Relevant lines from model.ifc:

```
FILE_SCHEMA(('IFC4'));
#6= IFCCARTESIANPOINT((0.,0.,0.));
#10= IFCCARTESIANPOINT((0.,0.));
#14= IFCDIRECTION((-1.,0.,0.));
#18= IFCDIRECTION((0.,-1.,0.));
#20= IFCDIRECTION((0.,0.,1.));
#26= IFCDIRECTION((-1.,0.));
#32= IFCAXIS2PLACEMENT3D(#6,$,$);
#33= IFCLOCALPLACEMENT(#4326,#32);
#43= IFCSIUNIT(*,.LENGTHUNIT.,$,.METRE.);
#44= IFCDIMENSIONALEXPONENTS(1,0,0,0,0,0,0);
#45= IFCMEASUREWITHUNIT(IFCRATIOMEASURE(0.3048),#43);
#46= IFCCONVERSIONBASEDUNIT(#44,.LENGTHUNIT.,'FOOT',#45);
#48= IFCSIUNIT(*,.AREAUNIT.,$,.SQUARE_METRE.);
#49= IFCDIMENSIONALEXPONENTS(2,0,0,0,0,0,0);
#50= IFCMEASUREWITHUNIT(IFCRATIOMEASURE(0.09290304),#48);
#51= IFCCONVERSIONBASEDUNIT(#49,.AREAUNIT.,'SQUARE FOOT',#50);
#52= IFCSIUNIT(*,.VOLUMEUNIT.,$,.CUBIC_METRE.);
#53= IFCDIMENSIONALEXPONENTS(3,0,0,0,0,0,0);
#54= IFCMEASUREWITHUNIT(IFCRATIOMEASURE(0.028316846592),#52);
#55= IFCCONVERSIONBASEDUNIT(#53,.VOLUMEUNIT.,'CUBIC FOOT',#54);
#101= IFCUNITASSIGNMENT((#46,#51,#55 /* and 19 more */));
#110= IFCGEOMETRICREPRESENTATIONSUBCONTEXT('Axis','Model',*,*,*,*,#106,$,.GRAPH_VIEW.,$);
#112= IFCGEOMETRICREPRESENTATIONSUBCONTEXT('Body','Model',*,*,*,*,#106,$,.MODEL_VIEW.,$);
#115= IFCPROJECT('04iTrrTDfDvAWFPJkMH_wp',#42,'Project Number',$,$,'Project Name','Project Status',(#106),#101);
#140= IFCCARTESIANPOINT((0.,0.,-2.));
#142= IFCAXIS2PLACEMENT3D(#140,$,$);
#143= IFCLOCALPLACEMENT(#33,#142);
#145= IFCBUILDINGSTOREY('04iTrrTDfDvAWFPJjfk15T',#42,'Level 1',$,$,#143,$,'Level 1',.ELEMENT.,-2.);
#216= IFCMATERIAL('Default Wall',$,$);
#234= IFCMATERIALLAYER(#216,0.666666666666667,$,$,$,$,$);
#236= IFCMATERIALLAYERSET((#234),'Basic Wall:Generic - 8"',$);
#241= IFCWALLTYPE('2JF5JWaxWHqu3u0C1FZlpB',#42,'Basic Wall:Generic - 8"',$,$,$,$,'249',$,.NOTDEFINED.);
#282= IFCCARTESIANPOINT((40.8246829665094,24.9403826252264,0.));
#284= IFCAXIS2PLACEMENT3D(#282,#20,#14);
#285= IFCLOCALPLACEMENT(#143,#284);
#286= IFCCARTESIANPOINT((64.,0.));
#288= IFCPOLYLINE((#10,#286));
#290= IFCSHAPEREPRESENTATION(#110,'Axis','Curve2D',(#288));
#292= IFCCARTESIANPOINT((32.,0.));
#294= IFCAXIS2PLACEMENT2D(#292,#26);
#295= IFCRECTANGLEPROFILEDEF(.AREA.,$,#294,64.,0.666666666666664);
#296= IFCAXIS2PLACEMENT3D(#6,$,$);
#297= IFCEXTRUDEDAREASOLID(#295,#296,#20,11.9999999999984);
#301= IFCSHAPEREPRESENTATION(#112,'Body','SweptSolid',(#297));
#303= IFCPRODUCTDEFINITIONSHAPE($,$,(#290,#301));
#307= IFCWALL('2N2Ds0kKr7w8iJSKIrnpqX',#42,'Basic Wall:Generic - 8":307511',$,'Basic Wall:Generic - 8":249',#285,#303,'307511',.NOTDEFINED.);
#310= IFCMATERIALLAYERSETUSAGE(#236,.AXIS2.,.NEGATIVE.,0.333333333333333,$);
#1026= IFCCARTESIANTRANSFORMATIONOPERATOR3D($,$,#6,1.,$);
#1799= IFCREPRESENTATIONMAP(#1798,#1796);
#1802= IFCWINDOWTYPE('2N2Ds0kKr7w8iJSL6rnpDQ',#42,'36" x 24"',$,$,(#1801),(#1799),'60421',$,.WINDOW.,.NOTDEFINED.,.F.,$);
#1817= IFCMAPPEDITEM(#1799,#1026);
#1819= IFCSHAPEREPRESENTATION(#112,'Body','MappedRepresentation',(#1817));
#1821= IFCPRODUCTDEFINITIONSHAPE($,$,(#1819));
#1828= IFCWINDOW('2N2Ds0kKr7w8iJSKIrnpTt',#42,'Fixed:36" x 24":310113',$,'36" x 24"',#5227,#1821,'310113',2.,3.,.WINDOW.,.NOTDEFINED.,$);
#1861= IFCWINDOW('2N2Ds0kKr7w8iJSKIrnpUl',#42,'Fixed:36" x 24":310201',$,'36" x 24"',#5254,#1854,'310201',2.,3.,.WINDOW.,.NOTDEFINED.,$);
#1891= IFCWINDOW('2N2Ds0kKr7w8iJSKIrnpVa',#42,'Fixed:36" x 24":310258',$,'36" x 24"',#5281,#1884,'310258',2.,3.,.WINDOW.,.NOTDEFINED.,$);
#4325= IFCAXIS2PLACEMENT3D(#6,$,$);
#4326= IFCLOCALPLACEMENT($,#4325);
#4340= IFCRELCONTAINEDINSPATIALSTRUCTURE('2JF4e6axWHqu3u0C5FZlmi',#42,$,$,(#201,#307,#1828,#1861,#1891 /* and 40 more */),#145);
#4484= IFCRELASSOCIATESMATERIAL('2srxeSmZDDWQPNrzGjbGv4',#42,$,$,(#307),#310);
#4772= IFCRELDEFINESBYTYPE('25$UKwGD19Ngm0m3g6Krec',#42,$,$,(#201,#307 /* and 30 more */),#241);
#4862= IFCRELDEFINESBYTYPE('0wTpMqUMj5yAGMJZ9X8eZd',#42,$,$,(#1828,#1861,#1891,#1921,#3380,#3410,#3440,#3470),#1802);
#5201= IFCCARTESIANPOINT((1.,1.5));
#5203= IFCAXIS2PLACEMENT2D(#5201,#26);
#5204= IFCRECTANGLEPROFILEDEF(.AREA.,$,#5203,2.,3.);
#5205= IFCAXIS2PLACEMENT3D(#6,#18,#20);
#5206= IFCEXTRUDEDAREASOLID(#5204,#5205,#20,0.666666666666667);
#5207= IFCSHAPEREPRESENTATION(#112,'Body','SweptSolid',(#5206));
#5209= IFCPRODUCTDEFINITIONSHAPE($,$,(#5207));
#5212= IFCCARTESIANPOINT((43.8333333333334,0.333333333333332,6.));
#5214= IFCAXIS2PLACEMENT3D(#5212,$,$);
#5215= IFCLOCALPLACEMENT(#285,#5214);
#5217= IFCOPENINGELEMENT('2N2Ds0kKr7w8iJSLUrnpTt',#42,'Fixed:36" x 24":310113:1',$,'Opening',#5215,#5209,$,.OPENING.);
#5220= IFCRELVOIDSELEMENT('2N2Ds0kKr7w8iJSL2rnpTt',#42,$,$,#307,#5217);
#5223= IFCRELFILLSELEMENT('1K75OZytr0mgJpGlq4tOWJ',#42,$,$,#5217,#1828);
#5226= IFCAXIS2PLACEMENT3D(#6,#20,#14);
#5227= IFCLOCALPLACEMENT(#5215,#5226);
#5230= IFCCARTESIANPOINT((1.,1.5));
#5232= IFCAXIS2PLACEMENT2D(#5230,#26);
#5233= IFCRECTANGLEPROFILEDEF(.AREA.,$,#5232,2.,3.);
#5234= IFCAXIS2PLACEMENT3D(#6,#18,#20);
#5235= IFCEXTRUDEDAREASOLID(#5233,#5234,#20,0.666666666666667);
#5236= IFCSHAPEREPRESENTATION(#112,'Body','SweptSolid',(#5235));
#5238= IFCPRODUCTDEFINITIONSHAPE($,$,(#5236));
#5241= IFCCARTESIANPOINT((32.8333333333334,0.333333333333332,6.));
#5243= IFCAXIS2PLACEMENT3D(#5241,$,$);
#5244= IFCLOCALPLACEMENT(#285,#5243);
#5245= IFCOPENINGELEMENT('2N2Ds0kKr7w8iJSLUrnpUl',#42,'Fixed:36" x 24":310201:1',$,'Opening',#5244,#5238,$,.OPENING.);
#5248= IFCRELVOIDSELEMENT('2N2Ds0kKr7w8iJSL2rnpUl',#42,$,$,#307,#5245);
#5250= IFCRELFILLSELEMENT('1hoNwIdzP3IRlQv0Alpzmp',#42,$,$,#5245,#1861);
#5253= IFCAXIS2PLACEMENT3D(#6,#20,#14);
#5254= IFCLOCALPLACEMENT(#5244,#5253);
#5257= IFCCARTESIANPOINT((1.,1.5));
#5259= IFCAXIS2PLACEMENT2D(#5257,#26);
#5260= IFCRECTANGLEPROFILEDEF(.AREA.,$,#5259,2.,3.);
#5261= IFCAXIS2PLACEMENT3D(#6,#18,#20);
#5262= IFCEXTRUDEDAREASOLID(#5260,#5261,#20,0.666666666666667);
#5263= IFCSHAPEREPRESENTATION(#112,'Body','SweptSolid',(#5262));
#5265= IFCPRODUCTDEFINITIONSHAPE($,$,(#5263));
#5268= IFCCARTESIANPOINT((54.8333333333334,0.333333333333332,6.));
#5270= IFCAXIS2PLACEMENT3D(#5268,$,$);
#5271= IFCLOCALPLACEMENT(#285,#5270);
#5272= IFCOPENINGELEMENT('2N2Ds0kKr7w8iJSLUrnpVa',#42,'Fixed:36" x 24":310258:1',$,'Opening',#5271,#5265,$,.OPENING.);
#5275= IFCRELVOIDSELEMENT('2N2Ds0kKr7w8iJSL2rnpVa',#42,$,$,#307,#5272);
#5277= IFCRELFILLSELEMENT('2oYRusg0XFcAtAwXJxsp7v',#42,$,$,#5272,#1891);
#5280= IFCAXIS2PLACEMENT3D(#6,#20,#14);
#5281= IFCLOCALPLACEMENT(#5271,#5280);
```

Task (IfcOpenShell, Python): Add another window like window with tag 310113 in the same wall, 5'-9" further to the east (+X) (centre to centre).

```python
import ifcopenshell
import ifcopenshell.api.feature
import ifcopenshell.api.geometry
import ifcopenshell.api.root
import ifcopenshell.geom
import ifcopenshell.util.element
import ifcopenshell.util.placement
import ifcopenshell.util.shape
import ifcopenshell.util.unit

model = ifcopenshell.open("model.ifc")
unit_scale = ifcopenshell.util.unit.calculate_unit_scale(model)
settings = ifcopenshell.geom.settings()


def volume(element):
    """Net volume in cubic metres, openings subtracted."""
    shape = ifcopenshell.geom.create_shape(settings, element)
    return ifcopenshell.util.shape.get_volume(shape.geometry)


def reuse_history(source, copy):
    """copy_class also copies each property set's owner history, people and application; keep the originals."""
    for rel in copy.IsDefinedBy:
        if rel.is_a("IfcRelDefinesByProperties") and (history := rel.RelatingPropertyDefinition.OwnerHistory):
            rel.RelatingPropertyDefinition.OwnerHistory = source.OwnerHistory
            ifcopenshell.util.element.remove_deep2(model, history)


window = model.by_id(1828)
opening = window.FillsVoids[0].RelatingOpeningElement
wall = opening.VoidsElements[0].RelatingBuildingElement
before = volume(wall)
shift = ifcopenshell.util.placement.get_local_placement(wall.ObjectPlacement)[:3, 0] * -69 * 0.0254 / unit_scale

# copy_class copies the void relationship, type, container and properties, but no geometry.
new_opening = ifcopenshell.api.root.copy_class(model, product=opening)
new_opening.Representation = ifcopenshell.util.element.copy_deep(
    model, opening.Representation, exclude=["IfcGeometricRepresentationContext", "IfcRepresentationMap"]
)
new_opening.Name = 'Fixed:36" x 24"'
new_window = ifcopenshell.api.root.copy_class(model, product=window)
new_window.Representation = ifcopenshell.util.element.copy_deep(
    model, window.Representation, exclude=["IfcGeometricRepresentationContext", "IfcRepresentationMap"]
)
new_window.Name = 'Fixed:36" x 24"'
new_window.Tag = None
reuse_history(window, new_window)
ifcopenshell.api.feature.add_filling(model, opening=new_opening, element=new_window)

for old, new in ((opening, new_opening), (window, new_window)):
    matrix = ifcopenshell.util.placement.get_local_placement(old.ObjectPlacement)
    matrix[:3, 3] += shift
    ifcopenshell.api.geometry.edit_object_placement(model, product=new, matrix=matrix, is_si=False)

after = volume(wall)

print(f"wall volume {before:.3f} -> {after:.3f} m3")

model.write("model_rev.ifc")
```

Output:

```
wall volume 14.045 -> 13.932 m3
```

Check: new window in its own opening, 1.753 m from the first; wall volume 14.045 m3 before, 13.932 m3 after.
